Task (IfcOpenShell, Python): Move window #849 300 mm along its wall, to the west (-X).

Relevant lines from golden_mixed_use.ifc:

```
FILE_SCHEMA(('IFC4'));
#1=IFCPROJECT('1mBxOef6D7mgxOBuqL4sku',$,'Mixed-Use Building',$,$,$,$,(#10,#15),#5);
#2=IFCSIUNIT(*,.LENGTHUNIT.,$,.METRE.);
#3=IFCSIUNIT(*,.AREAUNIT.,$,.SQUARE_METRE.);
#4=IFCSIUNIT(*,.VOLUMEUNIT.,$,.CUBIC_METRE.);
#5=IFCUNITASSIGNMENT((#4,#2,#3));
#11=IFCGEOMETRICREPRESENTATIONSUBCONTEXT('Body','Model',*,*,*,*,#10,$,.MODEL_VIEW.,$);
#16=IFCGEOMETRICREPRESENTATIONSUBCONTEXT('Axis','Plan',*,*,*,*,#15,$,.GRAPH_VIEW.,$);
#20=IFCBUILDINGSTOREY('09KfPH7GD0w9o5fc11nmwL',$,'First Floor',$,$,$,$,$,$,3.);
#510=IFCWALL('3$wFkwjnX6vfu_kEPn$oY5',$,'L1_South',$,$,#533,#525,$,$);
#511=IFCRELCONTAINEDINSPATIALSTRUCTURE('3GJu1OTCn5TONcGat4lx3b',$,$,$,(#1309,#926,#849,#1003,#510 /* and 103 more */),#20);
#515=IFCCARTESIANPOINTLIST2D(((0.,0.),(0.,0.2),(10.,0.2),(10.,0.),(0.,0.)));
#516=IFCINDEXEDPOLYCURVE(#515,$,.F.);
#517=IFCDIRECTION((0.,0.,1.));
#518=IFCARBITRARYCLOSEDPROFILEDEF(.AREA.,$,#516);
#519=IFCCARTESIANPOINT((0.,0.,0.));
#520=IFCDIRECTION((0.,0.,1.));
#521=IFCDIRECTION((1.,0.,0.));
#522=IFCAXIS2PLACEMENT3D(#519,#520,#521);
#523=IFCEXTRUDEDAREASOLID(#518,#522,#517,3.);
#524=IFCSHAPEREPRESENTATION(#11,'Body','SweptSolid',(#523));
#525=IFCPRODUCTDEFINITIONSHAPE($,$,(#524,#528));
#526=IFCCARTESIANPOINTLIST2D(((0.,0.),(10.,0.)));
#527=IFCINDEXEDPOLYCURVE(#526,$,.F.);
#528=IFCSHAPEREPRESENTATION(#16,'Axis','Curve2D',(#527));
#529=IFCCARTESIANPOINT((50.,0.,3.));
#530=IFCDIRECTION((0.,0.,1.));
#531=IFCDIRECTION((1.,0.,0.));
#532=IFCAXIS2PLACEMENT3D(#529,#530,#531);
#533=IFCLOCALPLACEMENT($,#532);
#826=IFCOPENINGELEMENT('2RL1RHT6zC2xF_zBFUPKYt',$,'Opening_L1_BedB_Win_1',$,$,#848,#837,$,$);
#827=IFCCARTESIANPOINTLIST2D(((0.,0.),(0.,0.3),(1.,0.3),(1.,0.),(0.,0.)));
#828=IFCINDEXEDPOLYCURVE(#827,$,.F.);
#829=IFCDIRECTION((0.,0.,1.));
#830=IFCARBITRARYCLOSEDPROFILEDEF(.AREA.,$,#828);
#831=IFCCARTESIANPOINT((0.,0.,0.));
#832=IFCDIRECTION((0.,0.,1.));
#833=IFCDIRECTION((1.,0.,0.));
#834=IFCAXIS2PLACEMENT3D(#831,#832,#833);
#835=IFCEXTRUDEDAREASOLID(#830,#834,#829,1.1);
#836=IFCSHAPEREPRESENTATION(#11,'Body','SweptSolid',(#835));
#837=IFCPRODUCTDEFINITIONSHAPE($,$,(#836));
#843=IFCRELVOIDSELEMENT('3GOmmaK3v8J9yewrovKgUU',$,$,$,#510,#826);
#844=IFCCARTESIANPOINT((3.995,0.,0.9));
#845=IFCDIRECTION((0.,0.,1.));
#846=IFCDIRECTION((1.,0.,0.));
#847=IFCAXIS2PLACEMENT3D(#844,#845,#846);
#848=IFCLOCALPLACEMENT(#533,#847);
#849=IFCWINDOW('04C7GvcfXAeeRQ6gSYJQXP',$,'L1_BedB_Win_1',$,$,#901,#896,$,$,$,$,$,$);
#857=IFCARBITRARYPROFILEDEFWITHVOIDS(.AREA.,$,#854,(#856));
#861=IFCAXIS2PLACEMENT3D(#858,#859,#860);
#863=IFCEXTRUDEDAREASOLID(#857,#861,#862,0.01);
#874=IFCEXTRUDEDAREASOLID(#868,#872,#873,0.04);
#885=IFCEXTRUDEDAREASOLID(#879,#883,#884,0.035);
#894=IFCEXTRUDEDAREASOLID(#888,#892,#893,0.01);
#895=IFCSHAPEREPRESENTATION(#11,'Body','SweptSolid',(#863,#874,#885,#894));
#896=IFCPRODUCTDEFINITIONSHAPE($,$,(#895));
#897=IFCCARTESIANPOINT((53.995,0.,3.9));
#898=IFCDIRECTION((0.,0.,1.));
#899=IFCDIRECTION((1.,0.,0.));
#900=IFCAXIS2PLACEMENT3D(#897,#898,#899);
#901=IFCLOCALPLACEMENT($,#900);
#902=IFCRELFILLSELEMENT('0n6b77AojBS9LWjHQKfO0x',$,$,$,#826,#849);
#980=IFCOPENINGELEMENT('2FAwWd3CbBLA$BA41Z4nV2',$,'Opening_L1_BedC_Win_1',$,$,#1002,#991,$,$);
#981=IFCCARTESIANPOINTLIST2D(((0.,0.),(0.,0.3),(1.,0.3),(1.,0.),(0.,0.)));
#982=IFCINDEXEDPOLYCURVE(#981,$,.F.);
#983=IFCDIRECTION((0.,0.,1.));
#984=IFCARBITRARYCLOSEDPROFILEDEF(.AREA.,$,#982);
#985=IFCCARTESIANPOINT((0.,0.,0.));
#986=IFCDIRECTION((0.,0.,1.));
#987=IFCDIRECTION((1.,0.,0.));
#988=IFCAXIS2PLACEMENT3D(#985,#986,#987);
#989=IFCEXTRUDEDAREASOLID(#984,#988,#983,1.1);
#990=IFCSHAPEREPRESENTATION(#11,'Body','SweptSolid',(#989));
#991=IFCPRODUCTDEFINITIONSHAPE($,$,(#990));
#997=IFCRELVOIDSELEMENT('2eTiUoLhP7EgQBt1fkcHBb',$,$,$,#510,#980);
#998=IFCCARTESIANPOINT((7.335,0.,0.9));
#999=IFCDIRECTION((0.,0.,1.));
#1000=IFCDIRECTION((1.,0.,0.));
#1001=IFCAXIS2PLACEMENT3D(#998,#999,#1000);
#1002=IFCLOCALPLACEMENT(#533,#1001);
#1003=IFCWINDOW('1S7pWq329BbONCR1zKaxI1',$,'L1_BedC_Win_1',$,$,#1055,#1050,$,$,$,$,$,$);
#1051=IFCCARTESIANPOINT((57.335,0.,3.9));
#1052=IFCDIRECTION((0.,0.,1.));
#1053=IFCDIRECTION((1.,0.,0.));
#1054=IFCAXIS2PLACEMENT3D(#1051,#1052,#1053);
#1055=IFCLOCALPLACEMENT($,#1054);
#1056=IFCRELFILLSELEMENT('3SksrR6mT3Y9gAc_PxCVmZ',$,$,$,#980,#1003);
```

```python
import ifcopenshell
import ifcopenshell.api.geometry
import ifcopenshell.util.placement
import ifcopenshell.util.unit

model = ifcopenshell.open("golden_mixed_use.ifc")
unit_scale = ifcopenshell.util.unit.calculate_unit_scale(model)

window = model.by_guid("04C7GvcfXAeeRQ6gSYJQXP")
opening = window.FillsVoids[0].RelatingOpeningElement
wall = opening.VoidsElements[0].RelatingBuildingElement

wall_matrix = ifcopenshell.util.placement.get_local_placement(wall.ObjectPlacement)
shift = wall_matrix[:3, 0] * -0.3 / unit_scale
before = ifcopenshell.util.placement.get_local_placement(window.ObjectPlacement)[:3, 3].copy()

# The window is not placed relative to its opening, so move both.
for product in (opening, window):
    matrix = ifcopenshell.util.placement.get_local_placement(product.ObjectPlacement)
    matrix[:3, 3] += shift
    ifcopenshell.api.geometry.edit_object_placement(model, product=product, matrix=matrix, is_si=False)

after = ifcopenshell.util.placement.get_local_placement(window.ObjectPlacement)[:3, 3]
print("window moved by", (after - before).round(3) + 0.0)

model.write("golden_mixed_use-out.ifc")
```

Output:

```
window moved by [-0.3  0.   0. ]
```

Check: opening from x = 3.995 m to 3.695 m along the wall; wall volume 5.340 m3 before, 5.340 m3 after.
